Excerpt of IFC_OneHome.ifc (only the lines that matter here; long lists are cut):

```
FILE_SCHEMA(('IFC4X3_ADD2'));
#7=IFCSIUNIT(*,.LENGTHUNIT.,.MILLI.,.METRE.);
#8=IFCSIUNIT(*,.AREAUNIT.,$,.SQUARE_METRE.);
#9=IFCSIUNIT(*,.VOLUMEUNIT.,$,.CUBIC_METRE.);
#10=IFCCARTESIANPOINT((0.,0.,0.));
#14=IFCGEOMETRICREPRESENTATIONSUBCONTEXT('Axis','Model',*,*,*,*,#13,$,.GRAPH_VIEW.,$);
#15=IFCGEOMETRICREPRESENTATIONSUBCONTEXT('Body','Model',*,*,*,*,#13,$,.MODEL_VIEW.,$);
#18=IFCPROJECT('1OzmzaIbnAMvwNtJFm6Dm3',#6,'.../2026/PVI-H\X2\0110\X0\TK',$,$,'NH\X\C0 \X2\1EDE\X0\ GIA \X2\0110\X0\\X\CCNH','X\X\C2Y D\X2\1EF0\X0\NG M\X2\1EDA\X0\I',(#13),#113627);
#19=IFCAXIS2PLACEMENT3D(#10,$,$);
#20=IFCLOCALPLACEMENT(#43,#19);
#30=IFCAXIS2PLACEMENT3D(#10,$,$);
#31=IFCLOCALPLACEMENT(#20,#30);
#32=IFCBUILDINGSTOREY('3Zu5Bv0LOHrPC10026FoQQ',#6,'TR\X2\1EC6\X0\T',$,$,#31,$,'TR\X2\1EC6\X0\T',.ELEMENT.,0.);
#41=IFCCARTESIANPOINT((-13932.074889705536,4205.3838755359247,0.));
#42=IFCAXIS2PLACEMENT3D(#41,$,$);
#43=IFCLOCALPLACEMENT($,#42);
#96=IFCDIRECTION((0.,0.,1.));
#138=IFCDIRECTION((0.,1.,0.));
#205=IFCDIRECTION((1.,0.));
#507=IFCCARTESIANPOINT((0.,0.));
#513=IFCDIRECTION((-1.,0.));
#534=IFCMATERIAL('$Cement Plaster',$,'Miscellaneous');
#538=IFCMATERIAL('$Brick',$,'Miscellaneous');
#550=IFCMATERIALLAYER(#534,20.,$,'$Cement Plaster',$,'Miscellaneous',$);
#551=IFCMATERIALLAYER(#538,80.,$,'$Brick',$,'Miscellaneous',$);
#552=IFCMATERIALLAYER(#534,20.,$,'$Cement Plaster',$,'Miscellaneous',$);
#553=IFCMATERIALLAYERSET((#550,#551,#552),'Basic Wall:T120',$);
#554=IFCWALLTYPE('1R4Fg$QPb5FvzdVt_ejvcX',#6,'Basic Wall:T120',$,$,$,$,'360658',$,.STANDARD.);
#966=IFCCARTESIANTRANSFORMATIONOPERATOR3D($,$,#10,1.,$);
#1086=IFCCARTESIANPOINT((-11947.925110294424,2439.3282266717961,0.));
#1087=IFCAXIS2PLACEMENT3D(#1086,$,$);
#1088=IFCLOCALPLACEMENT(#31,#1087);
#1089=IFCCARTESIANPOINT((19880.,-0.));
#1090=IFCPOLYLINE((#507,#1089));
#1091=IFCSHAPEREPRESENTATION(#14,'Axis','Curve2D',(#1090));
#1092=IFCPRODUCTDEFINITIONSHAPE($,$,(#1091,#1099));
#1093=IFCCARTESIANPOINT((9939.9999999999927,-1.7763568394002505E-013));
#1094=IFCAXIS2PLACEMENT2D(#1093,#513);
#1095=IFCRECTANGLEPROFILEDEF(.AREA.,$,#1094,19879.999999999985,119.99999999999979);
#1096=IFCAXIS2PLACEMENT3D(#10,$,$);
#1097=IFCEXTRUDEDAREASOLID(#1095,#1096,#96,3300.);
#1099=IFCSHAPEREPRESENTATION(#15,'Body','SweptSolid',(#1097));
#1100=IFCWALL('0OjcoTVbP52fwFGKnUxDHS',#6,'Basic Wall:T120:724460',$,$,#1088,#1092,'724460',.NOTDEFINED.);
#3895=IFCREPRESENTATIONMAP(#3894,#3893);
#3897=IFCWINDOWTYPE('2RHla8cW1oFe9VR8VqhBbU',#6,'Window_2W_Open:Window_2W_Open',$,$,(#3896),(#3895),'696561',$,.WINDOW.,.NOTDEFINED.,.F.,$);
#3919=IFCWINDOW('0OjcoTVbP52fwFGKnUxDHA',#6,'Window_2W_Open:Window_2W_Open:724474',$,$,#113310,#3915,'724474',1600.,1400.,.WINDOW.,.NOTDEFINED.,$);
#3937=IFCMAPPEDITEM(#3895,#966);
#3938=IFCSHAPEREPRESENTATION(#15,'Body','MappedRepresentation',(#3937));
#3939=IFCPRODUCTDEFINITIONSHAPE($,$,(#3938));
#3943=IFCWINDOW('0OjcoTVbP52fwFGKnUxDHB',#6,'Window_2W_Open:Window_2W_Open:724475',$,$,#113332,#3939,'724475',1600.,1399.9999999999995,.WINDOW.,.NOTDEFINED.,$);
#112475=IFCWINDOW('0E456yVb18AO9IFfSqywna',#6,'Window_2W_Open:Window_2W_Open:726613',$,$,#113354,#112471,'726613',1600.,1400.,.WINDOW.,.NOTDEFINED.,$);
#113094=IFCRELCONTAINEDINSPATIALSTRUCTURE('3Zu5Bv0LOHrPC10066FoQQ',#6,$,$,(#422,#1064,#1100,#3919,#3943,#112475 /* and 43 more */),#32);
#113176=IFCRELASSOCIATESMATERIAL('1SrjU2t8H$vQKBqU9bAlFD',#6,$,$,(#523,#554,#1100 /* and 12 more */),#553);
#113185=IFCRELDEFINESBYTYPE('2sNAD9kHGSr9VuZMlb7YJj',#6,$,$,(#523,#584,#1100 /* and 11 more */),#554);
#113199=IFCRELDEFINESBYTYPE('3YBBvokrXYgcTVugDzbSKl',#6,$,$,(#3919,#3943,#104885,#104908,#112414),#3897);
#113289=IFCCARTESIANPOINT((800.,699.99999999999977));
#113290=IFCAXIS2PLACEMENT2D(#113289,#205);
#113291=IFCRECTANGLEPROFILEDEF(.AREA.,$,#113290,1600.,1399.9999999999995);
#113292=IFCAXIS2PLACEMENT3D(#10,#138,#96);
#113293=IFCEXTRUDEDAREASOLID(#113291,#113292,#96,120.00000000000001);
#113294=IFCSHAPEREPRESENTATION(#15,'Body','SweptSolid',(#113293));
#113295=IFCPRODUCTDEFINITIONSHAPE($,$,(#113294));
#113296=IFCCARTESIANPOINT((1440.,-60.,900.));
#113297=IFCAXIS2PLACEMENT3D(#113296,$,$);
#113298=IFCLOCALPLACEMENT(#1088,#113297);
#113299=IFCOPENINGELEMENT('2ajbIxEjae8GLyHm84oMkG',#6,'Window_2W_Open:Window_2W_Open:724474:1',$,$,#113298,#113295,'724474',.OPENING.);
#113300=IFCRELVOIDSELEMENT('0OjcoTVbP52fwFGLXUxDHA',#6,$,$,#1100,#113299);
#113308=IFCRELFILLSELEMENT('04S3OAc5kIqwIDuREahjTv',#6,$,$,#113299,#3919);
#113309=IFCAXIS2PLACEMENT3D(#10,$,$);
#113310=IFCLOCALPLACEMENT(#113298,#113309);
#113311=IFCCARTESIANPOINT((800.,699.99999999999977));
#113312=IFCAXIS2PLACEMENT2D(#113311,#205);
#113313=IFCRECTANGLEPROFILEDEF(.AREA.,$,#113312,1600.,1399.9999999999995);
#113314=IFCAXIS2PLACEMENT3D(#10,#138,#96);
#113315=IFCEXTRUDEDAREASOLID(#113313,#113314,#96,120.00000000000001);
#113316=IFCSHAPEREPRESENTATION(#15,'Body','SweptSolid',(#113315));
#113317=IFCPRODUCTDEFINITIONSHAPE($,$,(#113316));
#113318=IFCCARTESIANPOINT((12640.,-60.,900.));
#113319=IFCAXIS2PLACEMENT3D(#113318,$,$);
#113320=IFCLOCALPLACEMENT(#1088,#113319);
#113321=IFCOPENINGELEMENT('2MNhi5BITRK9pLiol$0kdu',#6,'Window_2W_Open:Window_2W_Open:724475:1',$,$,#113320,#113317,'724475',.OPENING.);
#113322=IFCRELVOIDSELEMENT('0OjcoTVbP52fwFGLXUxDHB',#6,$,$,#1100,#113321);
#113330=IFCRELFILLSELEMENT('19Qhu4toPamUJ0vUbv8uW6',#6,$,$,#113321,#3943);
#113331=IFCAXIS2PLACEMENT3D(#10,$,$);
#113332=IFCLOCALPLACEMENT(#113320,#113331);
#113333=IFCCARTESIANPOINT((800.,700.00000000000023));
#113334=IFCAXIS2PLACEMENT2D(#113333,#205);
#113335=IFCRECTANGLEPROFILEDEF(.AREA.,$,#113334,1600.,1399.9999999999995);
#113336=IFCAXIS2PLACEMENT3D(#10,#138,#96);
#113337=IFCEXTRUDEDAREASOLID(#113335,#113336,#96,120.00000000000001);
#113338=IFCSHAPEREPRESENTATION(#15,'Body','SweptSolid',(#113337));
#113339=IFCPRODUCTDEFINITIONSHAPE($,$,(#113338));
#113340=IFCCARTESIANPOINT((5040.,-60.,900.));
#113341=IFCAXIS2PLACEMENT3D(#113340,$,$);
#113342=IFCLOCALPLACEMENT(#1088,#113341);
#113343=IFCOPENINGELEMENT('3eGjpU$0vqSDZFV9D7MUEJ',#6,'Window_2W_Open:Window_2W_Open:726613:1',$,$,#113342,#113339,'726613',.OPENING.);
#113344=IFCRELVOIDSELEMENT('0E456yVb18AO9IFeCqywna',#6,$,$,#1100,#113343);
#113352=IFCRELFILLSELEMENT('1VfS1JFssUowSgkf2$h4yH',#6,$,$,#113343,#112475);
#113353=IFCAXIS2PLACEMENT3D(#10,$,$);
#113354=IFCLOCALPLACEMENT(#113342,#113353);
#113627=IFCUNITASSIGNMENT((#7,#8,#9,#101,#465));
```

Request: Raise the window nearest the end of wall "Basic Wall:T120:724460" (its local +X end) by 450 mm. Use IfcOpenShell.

```python
import numpy as np
import ifcopenshell
import ifcopenshell.api.geometry
import ifcopenshell.util.placement
import ifcopenshell.util.unit

model = ifcopenshell.open("IFC_OneHome.ifc")
unit_scale = ifcopenshell.util.unit.calculate_unit_scale(model)

window = model.by_guid("0OjcoTVbP52fwFGKnUxDHB")
opening = window.FillsVoids[0].RelatingOpeningElement
dz = 0.45 / unit_scale

shift = np.array([0.0, 0.0, dz])
# The window is placed relative to its opening, so it follows when the opening moves.
matrix = ifcopenshell.util.placement.get_local_placement(opening.ObjectPlacement)
matrix[:3, 3] += shift
ifcopenshell.api.geometry.edit_object_placement(
    model, product=opening, matrix=matrix, is_si=False, should_transform_children=True
)

print(f"moved by {dz * unit_scale:+.3f} m")

model.write("IFC_OneHome_edited.ifc")
```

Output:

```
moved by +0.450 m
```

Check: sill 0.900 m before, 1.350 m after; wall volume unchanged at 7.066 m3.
